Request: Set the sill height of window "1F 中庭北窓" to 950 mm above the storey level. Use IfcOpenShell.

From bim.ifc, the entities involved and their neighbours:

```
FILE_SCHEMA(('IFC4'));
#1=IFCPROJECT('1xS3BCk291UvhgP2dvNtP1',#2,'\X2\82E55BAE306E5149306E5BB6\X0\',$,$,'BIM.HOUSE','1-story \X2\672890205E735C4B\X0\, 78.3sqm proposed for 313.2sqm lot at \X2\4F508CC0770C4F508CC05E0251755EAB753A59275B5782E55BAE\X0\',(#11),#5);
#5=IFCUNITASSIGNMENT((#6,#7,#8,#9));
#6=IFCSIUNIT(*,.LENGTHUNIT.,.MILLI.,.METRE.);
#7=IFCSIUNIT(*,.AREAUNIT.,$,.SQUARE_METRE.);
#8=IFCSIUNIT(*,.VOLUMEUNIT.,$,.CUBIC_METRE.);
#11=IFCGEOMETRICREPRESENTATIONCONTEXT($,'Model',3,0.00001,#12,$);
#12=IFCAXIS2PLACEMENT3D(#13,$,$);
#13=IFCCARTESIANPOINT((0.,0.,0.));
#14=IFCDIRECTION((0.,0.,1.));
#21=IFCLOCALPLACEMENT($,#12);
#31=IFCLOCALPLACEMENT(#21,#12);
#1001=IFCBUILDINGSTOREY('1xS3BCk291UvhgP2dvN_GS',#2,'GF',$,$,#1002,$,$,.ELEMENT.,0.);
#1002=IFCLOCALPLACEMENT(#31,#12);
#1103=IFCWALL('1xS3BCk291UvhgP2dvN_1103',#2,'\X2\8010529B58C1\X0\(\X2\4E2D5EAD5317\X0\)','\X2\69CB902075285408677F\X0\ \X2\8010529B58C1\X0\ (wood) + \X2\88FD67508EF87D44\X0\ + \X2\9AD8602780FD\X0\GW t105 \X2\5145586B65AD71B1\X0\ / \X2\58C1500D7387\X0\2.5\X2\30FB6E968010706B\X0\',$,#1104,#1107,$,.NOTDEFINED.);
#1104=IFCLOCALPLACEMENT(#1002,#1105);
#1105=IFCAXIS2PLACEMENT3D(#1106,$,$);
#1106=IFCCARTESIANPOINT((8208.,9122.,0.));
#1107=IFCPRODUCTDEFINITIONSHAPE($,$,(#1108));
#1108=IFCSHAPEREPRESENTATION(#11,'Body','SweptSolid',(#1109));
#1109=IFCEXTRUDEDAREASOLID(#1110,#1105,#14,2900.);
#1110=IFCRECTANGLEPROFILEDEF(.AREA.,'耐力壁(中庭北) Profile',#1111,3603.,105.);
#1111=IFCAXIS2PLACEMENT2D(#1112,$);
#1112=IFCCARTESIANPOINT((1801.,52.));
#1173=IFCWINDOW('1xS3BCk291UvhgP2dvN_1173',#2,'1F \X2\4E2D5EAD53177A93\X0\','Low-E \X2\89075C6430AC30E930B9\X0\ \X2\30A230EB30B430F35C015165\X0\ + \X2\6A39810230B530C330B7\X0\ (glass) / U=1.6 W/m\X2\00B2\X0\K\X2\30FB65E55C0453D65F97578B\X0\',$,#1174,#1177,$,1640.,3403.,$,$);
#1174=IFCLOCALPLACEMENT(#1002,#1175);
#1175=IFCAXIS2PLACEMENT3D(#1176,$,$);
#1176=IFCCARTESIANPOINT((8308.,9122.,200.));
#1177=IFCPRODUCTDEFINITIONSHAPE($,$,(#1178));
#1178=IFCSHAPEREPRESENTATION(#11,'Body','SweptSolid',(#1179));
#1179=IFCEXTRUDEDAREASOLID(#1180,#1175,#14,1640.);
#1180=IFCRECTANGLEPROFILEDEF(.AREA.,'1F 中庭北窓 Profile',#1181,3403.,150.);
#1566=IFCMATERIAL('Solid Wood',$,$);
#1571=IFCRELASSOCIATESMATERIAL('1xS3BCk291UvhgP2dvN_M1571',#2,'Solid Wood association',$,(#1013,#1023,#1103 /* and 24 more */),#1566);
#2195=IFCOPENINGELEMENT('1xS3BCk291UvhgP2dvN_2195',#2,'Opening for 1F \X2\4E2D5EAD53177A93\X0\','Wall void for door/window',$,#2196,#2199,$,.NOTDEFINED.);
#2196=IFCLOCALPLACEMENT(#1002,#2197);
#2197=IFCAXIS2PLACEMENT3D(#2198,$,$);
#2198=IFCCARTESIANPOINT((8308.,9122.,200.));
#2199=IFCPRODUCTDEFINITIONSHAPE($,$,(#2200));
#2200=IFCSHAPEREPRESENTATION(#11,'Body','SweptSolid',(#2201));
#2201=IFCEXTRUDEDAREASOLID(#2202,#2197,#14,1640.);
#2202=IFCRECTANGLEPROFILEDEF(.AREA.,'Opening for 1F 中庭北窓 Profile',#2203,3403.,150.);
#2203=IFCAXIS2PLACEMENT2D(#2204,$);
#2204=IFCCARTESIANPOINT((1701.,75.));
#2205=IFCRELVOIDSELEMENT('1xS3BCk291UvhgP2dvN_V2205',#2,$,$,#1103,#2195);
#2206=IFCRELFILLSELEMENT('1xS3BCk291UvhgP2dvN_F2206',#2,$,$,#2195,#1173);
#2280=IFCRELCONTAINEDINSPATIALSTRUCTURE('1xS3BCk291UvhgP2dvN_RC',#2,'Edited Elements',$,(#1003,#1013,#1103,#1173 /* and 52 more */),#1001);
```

```python
import numpy as np
import ifcopenshell
import ifcopenshell.api.geometry
import ifcopenshell.geom
import ifcopenshell.util.element
import ifcopenshell.util.placement
import ifcopenshell.util.shape
import ifcopenshell.util.unit

model = ifcopenshell.open("bim.ifc")
unit_scale = ifcopenshell.util.unit.calculate_unit_scale(model)

window = model.by_guid("1xS3BCk291UvhgP2dvN_1173")
opening = window.FillsVoids[0].RelatingOpeningElement
storey = ifcopenshell.util.element.get_container(window, ifc_class="IfcBuildingStorey")
level = ifcopenshell.util.placement.get_local_placement(storey.ObjectPlacement)[2, 3]

# The opening's origin need not be at the sill, so measure its lowest point.
shape = ifcopenshell.geom.create_shape(ifcopenshell.geom.settings(), opening)
bottom = ifcopenshell.util.shape.get_shape_bottom_elevation(shape, shape.geometry) / unit_scale
dz = level + 950.0 - bottom

shift = np.array([0.0, 0.0, dz])
# The window is not placed relative to its opening, so move both.
for product in (opening, window):
    matrix = ifcopenshell.util.placement.get_local_placement(product.ObjectPlacement)
    matrix[:3, 3] += shift
    ifcopenshell.api.geometry.edit_object_placement(model, product=product, matrix=matrix, is_si=False)

print(f"moved by {dz * unit_scale:+.3f} m")

model.write("bim_updated.ifc")
```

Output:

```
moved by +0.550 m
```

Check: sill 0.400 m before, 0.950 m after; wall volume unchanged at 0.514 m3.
